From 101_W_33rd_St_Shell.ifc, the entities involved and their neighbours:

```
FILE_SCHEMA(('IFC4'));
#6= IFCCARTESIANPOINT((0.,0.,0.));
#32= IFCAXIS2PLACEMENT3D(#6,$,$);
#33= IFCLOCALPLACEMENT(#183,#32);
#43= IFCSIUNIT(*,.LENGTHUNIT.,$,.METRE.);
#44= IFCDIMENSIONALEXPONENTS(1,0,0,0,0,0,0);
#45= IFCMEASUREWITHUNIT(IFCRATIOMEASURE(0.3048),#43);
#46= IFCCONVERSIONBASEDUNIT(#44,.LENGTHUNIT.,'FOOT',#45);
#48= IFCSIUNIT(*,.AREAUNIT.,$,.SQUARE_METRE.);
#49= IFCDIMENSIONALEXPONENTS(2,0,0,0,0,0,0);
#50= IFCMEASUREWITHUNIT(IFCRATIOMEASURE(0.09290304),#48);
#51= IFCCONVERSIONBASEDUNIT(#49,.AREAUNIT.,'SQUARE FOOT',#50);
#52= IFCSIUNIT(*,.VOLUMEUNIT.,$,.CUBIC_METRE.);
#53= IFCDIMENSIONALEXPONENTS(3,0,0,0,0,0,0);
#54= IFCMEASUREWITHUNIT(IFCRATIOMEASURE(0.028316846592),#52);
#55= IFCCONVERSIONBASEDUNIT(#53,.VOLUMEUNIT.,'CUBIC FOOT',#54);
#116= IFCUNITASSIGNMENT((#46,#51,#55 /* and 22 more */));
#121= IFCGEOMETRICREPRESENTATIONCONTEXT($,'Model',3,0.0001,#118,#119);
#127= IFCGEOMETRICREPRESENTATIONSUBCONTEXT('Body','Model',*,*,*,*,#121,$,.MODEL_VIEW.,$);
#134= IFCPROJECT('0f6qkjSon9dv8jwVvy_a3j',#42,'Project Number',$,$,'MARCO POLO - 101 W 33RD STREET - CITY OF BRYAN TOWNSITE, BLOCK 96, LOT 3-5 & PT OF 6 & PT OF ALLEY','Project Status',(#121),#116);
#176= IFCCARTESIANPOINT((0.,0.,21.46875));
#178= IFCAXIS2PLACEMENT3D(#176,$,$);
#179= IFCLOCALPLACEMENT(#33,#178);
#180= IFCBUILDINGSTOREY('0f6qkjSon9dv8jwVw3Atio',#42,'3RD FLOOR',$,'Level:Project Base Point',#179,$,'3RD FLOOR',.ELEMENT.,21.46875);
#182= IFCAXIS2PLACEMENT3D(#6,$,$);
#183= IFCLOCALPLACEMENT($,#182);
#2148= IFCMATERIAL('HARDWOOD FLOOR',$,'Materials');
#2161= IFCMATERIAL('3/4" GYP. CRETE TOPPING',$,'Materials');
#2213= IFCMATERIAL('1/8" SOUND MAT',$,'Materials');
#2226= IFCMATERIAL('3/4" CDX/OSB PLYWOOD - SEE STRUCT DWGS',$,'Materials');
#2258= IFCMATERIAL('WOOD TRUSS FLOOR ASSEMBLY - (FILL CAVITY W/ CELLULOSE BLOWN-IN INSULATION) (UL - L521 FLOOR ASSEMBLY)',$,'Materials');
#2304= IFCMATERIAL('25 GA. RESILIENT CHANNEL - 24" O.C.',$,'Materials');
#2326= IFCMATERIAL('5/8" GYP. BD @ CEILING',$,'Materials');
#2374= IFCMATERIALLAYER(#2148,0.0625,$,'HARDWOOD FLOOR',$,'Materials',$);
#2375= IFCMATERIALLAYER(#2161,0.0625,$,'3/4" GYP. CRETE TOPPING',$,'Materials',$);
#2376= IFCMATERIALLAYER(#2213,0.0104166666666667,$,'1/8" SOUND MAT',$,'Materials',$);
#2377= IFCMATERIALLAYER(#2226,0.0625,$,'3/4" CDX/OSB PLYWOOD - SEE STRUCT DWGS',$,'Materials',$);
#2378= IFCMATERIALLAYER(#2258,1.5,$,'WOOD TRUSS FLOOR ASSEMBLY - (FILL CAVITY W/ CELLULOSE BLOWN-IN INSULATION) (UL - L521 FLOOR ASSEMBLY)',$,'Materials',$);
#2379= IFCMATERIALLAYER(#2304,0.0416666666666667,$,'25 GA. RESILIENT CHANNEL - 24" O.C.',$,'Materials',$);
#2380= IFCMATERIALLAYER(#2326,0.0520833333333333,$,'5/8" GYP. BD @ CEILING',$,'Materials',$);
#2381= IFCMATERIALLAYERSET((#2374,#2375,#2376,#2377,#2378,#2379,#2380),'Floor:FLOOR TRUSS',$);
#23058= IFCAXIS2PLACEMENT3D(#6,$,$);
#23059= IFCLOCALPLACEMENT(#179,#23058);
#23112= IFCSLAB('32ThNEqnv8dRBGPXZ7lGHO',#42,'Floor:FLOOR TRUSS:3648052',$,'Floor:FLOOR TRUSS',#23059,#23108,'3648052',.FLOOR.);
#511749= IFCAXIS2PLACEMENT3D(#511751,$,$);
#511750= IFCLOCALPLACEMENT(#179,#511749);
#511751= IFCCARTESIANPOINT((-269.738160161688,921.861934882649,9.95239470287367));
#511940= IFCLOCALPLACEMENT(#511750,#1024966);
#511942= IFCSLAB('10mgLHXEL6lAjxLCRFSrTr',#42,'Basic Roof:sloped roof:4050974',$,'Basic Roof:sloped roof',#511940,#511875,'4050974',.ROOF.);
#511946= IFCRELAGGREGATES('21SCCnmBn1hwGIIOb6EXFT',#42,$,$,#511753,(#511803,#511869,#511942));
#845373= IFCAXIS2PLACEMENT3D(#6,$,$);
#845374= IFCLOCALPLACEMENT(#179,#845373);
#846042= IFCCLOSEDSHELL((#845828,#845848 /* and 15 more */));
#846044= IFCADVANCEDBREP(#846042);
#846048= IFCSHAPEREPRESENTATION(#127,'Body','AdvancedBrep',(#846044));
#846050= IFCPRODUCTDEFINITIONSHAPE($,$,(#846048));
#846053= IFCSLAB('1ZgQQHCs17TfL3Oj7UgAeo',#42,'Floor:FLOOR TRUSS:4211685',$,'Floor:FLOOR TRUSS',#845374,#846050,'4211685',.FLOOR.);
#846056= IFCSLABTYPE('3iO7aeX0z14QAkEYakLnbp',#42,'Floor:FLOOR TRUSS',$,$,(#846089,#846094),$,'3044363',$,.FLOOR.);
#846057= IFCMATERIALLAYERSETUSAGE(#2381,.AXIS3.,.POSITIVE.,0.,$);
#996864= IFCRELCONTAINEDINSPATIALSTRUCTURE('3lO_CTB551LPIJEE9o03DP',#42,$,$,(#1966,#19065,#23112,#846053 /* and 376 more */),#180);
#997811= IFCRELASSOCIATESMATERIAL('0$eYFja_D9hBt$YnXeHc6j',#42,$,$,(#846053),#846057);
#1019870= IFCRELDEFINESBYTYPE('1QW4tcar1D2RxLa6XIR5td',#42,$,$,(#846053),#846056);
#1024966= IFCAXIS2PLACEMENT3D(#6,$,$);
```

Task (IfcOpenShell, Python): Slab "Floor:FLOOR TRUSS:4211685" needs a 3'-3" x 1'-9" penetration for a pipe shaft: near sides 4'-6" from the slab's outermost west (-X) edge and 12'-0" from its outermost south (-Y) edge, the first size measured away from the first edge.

```python
import numpy as np
import ifcopenshell
import ifcopenshell.api.feature
import ifcopenshell.api.geometry
import ifcopenshell.api.root
import ifcopenshell.geom
import ifcopenshell.util.placement
import ifcopenshell.util.representation
import ifcopenshell.util.shape
import ifcopenshell.util.unit

model = ifcopenshell.open("101_W_33rd_St_Shell.ifc")
unit_scale = ifcopenshell.util.unit.calculate_unit_scale(model)
settings = ifcopenshell.geom.settings()


def volume(element):
    """Net volume in cubic metres, openings subtracted."""
    shape = ifcopenshell.geom.create_shape(settings, element)
    return ifcopenshell.util.shape.get_volume(shape.geometry)


slab = model.by_guid("1ZgQQHCs17TfL3Oj7UgAeo")
before = volume(slab)

# Extent in the slab's own axes, in metres. The edges named are its -X and -Y sides.
slab_shape = ifcopenshell.geom.create_shape(settings, slab)
vertices = ifcopenshell.util.shape.get_vertices(slab_shape.geometry)
x_min, y_min, bottom = vertices.min(axis=0)
top = vertices[:, 2].max()

opening = ifcopenshell.api.root.create_entity(model, ifc_class="IfcOpeningElement", name="Pipe shaft opening", predefined_type="OPENING")
context = ifcopenshell.util.representation.get_context(model, "Model", "Body", "MODEL_VIEW")
width, depth = 0.9906, 0.5334
outline = [(0.0, 0.0), (width, 0.0), (width, depth), (0.0, depth), (0.0, 0.0)]
# Overshoot both faces by 50 mm so the cut is clean.
shape = ifcopenshell.api.geometry.add_slab_representation(
    model, context=context, depth=top - bottom + 0.1, polyline=outline
)
ifcopenshell.api.geometry.assign_representation(model, product=opening, representation=shape)

matrix = ifcopenshell.util.placement.get_local_placement(slab.ObjectPlacement)
matrix[:, 3] = matrix @ np.append(np.array([x_min + 1.3716, y_min + 3.6576, bottom - 0.05]) / unit_scale, 1.0)
ifcopenshell.api.geometry.edit_object_placement(model, product=opening, matrix=matrix, is_si=False)
ifcopenshell.api.feature.add_feature(model, feature=opening, element=slab)

after = volume(slab)

print(f"slab volume {before:.3f} -> {after:.3f} m3")

model.write("101_W_33rd_St_Shell_v2.ifc")
```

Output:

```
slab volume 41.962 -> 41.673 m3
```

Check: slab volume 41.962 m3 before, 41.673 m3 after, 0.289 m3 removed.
